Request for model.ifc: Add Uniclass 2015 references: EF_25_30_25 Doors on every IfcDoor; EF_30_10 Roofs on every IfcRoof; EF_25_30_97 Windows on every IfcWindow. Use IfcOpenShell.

First a look at what the model holds.

```python
import ifcopenshell

model = ifcopenshell.open("model.ifc")
print(model.schema)
print("classifications:", [c.Name for c in model.by_type("IfcClassification")])
for ifc_class in ("IfcDoor", "IfcRoof", "IfcStair", "IfcWall", "IfcWindow"):
    print(ifc_class, len(model.by_type(ifc_class)))
```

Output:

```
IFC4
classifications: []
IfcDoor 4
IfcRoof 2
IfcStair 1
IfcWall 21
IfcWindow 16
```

```python
import ifcopenshell
import ifcopenshell.api.classification

model = ifcopenshell.open("model.ifc")

system = ifcopenshell.api.classification.add_classification(model, classification="Uniclass 2015")

codes = {
    "IfcDoor": ("EF_25_30_25", "Doors"),
    "IfcRoof": ("EF_30_10", "Roofs"),
    "IfcWindow": ("EF_25_30_97", "Windows"),
}
for ifc_class, (code, name) in codes.items():
    products = model.by_type(ifc_class)
    ifcopenshell.api.classification.add_reference(
        model, products=products, classification=system, identification=code, name=name
    )
    print(code, len(products))

model.write("model_v2.ifc")
```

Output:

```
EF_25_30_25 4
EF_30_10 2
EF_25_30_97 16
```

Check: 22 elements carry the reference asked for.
